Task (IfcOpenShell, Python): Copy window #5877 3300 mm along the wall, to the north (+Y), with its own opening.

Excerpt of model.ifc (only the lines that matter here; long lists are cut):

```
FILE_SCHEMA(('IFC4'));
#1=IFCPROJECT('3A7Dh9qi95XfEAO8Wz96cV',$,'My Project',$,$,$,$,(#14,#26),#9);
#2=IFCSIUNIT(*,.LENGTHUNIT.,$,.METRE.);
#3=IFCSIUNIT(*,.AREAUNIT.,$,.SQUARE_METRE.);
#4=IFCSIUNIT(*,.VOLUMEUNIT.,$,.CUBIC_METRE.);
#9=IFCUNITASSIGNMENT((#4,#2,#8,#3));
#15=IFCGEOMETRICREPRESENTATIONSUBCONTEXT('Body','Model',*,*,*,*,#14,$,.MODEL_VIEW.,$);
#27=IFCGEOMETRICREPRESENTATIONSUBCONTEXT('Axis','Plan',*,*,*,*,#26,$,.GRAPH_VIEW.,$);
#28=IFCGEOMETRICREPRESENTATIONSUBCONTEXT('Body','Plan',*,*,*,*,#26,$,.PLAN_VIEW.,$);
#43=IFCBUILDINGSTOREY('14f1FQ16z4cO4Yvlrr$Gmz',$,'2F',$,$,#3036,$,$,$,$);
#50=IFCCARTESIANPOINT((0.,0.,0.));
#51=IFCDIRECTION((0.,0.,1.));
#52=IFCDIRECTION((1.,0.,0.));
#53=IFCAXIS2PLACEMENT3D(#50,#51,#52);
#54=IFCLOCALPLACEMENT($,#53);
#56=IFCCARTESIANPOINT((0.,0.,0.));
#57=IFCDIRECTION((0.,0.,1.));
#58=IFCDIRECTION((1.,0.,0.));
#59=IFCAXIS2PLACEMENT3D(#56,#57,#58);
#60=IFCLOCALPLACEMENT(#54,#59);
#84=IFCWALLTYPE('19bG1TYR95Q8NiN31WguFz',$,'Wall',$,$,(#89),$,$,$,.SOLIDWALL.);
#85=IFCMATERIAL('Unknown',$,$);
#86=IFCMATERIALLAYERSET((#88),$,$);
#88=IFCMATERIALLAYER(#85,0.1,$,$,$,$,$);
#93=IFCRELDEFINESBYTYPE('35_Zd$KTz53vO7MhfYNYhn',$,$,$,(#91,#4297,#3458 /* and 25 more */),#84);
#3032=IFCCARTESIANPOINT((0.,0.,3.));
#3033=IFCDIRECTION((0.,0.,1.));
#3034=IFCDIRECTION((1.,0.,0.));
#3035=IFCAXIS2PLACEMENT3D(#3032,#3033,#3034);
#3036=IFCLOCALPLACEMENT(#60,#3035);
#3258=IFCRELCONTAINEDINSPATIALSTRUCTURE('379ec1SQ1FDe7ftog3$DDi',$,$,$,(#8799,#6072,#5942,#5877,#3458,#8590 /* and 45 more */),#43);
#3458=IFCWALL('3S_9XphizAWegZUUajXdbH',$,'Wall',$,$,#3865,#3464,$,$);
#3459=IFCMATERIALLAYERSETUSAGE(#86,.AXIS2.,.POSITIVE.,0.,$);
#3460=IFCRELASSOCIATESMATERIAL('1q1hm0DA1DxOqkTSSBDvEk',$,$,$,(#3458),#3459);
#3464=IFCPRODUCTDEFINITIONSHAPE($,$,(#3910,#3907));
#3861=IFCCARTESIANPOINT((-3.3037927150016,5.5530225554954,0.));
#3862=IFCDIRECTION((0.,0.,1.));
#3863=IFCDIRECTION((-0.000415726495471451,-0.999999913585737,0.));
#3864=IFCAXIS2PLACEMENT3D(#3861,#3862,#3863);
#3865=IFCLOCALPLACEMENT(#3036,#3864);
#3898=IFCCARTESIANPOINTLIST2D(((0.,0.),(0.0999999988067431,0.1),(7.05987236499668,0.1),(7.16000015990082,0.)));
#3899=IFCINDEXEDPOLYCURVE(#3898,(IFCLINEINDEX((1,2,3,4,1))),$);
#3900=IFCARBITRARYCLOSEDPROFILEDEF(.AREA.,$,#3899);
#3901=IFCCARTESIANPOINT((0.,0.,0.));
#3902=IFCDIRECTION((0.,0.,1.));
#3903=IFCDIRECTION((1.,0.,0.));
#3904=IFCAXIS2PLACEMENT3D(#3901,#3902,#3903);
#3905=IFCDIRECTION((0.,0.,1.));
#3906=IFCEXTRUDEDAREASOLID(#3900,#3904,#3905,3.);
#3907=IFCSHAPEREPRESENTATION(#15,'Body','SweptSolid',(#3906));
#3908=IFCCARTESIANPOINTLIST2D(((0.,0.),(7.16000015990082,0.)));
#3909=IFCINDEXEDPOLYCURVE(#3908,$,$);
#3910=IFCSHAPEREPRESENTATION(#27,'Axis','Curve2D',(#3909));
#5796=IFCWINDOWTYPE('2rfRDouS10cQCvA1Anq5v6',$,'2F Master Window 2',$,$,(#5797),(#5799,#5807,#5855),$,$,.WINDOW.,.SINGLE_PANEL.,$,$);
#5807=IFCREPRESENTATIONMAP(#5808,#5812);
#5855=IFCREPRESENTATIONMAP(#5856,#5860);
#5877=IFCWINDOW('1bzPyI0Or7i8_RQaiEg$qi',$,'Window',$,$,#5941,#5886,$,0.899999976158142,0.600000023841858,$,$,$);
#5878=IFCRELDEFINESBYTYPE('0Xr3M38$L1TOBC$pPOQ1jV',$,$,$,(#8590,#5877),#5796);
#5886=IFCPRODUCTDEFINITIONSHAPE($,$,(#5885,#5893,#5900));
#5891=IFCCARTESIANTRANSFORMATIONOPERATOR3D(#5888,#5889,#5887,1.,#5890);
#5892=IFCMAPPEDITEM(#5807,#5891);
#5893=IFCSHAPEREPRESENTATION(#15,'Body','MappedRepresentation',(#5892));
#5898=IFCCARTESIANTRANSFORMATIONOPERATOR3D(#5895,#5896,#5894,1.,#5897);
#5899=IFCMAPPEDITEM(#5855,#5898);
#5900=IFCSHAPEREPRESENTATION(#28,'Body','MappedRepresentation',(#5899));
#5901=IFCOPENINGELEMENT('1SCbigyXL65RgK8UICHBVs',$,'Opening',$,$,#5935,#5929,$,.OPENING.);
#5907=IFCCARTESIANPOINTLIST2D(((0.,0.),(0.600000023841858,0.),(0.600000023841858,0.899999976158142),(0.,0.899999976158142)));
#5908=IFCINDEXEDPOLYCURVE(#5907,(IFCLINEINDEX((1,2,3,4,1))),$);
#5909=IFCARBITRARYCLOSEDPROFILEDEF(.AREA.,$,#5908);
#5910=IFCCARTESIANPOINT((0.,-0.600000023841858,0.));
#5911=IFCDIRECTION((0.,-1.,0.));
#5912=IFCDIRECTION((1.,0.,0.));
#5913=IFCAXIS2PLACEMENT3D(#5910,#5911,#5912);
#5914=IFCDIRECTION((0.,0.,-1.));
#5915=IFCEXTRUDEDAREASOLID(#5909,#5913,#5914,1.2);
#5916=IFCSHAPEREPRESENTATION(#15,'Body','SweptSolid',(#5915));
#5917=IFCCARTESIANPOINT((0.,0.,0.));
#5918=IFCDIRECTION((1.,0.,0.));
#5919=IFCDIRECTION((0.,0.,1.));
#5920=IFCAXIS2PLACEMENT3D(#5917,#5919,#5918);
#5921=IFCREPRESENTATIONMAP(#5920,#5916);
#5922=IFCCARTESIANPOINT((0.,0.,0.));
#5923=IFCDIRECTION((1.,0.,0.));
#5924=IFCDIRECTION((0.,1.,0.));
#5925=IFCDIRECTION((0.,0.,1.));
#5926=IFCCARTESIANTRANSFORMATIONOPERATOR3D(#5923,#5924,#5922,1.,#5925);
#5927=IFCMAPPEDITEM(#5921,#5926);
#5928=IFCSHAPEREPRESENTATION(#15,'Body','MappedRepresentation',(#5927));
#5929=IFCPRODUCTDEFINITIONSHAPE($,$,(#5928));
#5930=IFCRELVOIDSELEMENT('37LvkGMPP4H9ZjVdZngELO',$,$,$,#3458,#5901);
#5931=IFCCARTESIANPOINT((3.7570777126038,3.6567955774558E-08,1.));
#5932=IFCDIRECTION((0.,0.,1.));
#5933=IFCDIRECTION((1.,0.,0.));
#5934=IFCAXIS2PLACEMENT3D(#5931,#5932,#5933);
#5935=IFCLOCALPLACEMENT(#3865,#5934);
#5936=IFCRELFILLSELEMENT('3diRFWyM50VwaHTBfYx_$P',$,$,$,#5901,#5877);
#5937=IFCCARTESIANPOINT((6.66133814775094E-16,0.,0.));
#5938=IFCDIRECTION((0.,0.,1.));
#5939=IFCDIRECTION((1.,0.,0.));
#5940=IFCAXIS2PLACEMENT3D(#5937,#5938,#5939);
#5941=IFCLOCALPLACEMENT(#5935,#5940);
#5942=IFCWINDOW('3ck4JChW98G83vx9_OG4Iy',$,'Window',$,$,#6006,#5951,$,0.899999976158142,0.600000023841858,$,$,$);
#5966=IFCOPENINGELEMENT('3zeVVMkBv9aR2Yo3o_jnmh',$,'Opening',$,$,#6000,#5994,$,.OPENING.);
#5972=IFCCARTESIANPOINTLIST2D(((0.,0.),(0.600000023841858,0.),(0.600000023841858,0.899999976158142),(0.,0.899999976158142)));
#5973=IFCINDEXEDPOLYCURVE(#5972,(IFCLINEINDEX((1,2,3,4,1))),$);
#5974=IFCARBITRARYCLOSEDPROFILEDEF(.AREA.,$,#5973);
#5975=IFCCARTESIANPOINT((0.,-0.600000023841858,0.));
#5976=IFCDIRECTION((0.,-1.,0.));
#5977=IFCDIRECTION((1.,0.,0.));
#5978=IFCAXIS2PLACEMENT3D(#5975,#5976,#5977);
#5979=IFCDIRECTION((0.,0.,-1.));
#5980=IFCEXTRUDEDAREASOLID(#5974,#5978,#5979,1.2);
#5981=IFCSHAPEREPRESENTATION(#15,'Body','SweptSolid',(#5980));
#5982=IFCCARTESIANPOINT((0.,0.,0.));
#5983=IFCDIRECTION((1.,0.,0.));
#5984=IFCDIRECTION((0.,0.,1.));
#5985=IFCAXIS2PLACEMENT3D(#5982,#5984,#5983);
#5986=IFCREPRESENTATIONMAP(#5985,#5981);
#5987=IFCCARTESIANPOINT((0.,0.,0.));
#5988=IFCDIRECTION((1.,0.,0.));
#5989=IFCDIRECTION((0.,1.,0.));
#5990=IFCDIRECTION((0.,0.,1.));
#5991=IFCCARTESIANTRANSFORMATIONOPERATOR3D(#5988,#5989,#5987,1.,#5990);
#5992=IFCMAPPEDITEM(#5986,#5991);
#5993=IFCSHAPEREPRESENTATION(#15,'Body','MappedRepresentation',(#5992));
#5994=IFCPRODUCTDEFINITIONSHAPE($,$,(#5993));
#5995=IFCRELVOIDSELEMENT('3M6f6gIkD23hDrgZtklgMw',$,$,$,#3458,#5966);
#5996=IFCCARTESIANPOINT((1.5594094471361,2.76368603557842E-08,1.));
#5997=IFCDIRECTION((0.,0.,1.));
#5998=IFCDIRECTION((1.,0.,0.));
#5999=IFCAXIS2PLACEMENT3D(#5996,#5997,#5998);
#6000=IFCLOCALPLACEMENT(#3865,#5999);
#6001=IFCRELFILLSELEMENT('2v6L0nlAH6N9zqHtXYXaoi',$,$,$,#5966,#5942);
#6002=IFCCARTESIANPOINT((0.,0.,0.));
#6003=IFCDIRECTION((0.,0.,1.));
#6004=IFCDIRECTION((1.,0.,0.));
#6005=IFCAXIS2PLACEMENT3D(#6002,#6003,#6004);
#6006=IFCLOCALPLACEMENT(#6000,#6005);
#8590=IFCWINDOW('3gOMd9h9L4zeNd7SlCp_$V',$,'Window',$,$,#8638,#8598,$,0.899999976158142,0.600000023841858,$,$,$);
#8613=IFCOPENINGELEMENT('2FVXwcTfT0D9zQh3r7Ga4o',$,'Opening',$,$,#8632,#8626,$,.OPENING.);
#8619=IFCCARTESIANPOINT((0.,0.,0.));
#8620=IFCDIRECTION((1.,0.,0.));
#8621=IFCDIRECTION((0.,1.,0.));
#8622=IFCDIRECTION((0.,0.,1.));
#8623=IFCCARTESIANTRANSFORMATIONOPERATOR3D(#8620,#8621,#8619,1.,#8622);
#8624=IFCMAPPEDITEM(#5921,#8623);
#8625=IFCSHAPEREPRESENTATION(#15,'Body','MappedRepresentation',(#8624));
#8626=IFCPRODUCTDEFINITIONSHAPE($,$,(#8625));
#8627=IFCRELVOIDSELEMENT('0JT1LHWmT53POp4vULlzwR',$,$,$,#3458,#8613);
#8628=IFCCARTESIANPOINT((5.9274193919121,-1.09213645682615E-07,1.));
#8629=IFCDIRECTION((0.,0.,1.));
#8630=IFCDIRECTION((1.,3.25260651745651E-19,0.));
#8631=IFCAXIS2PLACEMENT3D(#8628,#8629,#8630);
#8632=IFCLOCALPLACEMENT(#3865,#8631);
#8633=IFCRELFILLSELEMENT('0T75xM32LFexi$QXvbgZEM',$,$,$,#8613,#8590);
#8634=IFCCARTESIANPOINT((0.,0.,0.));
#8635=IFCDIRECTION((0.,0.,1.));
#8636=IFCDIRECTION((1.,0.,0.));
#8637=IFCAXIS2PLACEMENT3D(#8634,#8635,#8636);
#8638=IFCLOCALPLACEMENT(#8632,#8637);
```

```python
import ifcopenshell
import ifcopenshell.api.feature
import ifcopenshell.api.geometry
import ifcopenshell.api.root
import ifcopenshell.geom
import ifcopenshell.util.element
import ifcopenshell.util.placement
import ifcopenshell.util.shape
import ifcopenshell.util.unit

model = ifcopenshell.open("model.ifc")
unit_scale = ifcopenshell.util.unit.calculate_unit_scale(model)
settings = ifcopenshell.geom.settings()


def volume(element):
    """Net volume in cubic metres, openings subtracted."""
    shape = ifcopenshell.geom.create_shape(settings, element)
    return ifcopenshell.util.shape.get_volume(shape.geometry)


window = model.by_id(5877)
opening = window.FillsVoids[0].RelatingOpeningElement
wall = opening.VoidsElements[0].RelatingBuildingElement
before = volume(wall)
shift = ifcopenshell.util.placement.get_local_placement(wall.ObjectPlacement)[:3, 0] * -3.3 / unit_scale

# copy_class copies the void relationship, type, container and properties, but no geometry.
new_opening = ifcopenshell.api.root.copy_class(model, product=opening)
new_opening.Representation = ifcopenshell.util.element.copy_deep(
    model, opening.Representation, exclude=["IfcGeometricRepresentationContext", "IfcRepresentationMap"]
)
new_window = ifcopenshell.api.root.copy_class(model, product=window)
new_window.Representation = ifcopenshell.util.element.copy_deep(
    model, window.Representation, exclude=["IfcGeometricRepresentationContext", "IfcRepresentationMap"]
)
ifcopenshell.api.feature.add_filling(model, opening=new_opening, element=new_window)

for old, new in ((opening, new_opening), (window, new_window)):
    matrix = ifcopenshell.util.placement.get_local_placement(old.ObjectPlacement)
    matrix[:3, 3] += shift
    ifcopenshell.api.geometry.edit_object_placement(model, product=new, matrix=matrix, is_si=False)

after = volume(wall)

print(f"wall volume {before:.3f} -> {after:.3f} m3")

model.write("model_v2.ifc")
```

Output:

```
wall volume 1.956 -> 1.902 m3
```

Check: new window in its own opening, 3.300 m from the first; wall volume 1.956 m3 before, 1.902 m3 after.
